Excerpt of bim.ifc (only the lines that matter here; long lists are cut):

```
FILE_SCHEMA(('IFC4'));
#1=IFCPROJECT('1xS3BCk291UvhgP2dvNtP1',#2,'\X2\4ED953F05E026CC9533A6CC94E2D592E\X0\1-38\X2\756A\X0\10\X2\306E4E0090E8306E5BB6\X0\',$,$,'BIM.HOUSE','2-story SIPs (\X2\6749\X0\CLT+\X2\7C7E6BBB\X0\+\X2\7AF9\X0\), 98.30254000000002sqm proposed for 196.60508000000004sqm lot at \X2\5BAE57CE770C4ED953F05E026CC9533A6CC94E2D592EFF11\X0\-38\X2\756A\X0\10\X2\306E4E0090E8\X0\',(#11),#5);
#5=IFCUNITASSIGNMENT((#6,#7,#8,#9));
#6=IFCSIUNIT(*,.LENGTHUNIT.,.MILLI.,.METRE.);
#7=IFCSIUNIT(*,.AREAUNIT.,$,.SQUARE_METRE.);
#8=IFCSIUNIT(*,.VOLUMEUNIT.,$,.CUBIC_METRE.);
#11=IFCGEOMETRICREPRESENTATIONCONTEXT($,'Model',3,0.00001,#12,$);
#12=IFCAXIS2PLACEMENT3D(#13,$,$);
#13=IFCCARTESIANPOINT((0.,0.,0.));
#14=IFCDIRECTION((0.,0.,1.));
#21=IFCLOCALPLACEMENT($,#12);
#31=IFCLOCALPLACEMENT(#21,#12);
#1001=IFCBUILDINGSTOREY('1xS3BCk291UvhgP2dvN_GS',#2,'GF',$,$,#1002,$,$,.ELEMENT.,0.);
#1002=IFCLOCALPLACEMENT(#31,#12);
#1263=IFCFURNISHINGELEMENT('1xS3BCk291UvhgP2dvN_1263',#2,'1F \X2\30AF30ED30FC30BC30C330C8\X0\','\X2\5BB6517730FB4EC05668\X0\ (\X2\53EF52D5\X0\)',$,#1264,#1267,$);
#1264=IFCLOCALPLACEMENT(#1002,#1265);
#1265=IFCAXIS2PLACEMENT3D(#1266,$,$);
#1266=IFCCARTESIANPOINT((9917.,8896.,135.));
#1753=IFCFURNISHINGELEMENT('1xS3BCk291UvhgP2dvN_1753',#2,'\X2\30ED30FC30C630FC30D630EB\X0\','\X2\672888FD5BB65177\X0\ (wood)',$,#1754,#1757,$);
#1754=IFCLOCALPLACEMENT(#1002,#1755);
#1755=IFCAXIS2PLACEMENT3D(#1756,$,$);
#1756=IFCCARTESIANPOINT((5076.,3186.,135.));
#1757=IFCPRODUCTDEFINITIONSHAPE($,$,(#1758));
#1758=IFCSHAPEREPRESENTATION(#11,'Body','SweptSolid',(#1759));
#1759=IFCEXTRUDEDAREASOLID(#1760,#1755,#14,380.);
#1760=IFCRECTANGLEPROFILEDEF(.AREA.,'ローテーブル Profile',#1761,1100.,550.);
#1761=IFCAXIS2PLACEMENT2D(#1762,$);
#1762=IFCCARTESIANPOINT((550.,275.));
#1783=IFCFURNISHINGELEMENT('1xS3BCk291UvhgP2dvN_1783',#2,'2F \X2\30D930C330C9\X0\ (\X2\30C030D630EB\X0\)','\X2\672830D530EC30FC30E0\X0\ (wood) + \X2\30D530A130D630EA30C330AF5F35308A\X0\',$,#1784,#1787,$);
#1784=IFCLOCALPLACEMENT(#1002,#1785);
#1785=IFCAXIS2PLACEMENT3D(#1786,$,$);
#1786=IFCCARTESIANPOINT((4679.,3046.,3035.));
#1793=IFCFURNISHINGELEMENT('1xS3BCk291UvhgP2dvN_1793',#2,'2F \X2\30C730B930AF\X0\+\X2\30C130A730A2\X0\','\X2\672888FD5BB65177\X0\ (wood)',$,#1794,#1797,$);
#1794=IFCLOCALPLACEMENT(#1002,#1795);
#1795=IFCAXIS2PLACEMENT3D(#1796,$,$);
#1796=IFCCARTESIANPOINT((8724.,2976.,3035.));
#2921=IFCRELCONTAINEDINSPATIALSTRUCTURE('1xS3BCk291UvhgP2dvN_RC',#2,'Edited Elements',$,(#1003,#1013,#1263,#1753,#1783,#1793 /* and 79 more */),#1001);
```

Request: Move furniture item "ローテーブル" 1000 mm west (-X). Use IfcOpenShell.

```python
import ifcopenshell
import ifcopenshell.api.geometry
import ifcopenshell.util.placement
import ifcopenshell.util.unit

model = ifcopenshell.open("bim.ifc")
unit_scale = ifcopenshell.util.unit.calculate_unit_scale(model)

item = model.by_guid("1xS3BCk291UvhgP2dvN_1753")
matrix = ifcopenshell.util.placement.get_local_placement(item.ObjectPlacement)
matrix[0, 3] -= 1 / unit_scale
ifcopenshell.api.geometry.edit_object_placement(model, product=item, matrix=matrix, is_si=False)

print(ifcopenshell.util.placement.get_local_placement(item.ObjectPlacement).round(3) + 0.0)

model.write("bim_v2.ifc")
```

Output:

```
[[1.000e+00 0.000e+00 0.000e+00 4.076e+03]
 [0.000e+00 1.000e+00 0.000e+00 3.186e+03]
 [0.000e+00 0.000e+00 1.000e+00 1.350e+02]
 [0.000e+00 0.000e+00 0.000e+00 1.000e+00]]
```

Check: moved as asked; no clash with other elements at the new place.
